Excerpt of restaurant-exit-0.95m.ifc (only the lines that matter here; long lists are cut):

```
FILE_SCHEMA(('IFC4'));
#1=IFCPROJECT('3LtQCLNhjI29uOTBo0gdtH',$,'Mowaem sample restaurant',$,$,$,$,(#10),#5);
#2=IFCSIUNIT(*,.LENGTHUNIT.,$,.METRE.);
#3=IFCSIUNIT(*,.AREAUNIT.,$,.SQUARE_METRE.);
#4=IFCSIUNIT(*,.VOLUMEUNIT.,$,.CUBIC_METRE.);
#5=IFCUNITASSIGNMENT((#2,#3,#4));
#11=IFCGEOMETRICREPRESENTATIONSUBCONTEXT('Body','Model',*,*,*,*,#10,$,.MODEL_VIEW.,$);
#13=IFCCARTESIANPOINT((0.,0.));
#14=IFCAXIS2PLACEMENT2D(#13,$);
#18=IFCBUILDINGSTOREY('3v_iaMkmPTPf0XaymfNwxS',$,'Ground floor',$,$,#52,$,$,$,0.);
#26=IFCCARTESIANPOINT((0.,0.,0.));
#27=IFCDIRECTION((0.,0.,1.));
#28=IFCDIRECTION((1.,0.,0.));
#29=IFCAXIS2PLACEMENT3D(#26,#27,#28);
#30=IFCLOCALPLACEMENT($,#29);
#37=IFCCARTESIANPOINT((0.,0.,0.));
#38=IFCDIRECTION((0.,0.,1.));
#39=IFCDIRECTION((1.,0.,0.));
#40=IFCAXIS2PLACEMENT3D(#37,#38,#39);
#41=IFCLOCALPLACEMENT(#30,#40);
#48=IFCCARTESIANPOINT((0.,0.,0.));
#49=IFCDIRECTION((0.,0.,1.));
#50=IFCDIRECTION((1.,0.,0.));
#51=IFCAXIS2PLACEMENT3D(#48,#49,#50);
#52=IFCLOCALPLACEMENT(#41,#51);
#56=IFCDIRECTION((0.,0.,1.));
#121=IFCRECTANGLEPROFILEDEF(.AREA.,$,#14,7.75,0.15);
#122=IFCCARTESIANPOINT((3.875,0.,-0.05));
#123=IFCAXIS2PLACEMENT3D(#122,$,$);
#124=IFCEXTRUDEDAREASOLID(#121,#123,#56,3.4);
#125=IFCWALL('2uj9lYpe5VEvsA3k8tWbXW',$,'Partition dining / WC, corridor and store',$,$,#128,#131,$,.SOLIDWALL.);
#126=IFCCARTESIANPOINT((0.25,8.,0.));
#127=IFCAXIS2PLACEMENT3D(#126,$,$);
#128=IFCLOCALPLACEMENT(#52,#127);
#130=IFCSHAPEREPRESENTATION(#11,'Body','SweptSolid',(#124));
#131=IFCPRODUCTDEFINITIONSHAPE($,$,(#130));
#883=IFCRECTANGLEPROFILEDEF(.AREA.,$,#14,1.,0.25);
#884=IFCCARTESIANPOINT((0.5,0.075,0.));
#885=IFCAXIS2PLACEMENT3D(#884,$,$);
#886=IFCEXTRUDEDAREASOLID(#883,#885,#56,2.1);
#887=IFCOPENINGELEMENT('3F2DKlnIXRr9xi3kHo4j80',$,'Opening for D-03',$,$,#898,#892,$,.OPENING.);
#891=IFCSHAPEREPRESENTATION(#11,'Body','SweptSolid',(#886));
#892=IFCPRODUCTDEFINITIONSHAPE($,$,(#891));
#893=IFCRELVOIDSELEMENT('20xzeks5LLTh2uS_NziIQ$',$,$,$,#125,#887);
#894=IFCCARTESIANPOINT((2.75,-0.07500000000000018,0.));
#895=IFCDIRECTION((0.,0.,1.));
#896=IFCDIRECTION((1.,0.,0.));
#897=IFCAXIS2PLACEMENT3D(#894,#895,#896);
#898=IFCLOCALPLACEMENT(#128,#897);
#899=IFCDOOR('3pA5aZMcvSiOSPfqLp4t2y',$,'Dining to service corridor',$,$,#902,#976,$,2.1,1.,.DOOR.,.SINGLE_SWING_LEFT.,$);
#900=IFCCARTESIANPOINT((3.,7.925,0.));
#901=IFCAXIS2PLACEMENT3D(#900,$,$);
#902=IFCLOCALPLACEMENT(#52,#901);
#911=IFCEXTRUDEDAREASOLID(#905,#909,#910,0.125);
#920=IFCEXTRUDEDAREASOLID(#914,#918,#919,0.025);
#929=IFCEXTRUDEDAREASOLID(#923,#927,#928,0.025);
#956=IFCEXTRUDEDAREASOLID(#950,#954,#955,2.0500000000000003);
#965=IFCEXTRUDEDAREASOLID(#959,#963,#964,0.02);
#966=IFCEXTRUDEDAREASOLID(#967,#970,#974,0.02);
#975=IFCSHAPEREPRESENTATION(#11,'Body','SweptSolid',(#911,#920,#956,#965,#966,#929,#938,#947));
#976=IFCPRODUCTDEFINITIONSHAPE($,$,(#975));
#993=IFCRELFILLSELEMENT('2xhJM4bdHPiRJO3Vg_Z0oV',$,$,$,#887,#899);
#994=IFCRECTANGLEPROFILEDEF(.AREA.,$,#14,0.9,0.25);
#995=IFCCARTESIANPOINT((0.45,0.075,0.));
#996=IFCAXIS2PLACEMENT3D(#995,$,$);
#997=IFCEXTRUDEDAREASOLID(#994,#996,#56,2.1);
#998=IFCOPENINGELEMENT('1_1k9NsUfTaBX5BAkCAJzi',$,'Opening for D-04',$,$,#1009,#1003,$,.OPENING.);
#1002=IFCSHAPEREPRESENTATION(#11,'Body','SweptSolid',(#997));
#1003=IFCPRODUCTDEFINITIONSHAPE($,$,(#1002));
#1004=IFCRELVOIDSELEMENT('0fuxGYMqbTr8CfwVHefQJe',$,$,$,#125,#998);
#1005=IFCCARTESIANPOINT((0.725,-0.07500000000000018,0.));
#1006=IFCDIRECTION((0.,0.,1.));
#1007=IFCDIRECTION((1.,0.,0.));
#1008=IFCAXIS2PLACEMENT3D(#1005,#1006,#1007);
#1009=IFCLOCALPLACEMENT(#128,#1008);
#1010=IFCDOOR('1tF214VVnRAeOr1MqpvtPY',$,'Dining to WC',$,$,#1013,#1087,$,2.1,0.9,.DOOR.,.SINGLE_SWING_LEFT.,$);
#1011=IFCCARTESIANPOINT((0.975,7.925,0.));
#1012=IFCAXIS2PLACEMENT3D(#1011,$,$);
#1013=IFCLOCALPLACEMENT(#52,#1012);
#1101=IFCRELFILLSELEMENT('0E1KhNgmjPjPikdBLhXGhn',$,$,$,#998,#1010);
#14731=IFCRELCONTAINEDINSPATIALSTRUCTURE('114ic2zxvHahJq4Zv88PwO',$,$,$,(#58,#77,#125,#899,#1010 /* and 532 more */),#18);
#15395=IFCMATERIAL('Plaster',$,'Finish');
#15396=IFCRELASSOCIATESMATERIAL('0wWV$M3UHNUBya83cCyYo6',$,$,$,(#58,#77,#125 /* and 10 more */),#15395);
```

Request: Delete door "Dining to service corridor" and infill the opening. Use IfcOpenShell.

```python
import ifcopenshell
import ifcopenshell.api.feature
import ifcopenshell.api.root
import ifcopenshell.geom
import ifcopenshell.util.shape

model = ifcopenshell.open("restaurant-exit-0.95m.ifc")
settings = ifcopenshell.geom.settings()


def volume(element):
    """Net volume in cubic metres, openings subtracted."""
    shape = ifcopenshell.geom.create_shape(settings, element)
    return ifcopenshell.util.shape.get_volume(shape.geometry)


door = model.by_guid("3pA5aZMcvSiOSPfqLp4t2y")
opening = door.FillsVoids[0].RelatingOpeningElement
wall = opening.VoidsElements[0].RelatingBuildingElement
before = volume(wall)

ifcopenshell.api.root.remove_product(model, product=door)
ifcopenshell.api.feature.remove_feature(model, feature=opening)

after = volume(wall)

print(f"wall volume {before:.3f} -> {after:.3f} m3")

model.write("restaurant-exit-0.95m_v2.ifc")
```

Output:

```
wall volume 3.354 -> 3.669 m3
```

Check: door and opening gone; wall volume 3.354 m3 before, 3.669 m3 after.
